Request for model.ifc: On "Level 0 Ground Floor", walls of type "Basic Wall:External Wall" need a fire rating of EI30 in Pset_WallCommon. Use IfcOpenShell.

First a look at what the model holds.

```python
import ifcopenshell
import ifcopenshell.util.element

model = ifcopenshell.open("model.ifc")
print(model.schema)
storey = next(s for s in model.by_type("IfcBuildingStorey") if s.Name == "Level 0 Ground Floor")
walls = [e for e in ifcopenshell.util.element.get_decomposition(storey) if e.is_a("IfcWall")]
seen = {}
for e in walls:
    element_type = ifcopenshell.util.element.get_type(e)
    key = (element_type.Name if element_type != e and element_type else None, ifcopenshell.util.element.get_pset(e, "Pset_WallCommon", "FireRating"))
    seen[key] = seen.get(key, 0) + 1
for (name, value), count in sorted(seen.items(), key=str):
    print(count, "x", name, "|", value)
```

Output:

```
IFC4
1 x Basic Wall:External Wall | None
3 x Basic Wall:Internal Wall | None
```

```python
import ifcopenshell
import ifcopenshell.api.pset
import ifcopenshell.util.element

model = ifcopenshell.open("model.ifc")

storey = next(s for s in model.by_type("IfcBuildingStorey") if s.Name == "Level 0 Ground Floor")
walls = [e for e in ifcopenshell.util.element.get_decomposition(storey) if e.is_a("IfcWall")]

count = 0
for e in walls:
    element_type = ifcopenshell.util.element.get_type(e)
    if element_type in (None, e) or element_type.Name != "Basic Wall:External Wall":
        continue
    # add_pset returns the element's existing set when there is one.
    pset = ifcopenshell.api.pset.add_pset(model, product=e, name="Pset_WallCommon")
    ifcopenshell.api.pset.edit_pset(model, pset=pset, properties={"FireRating": "EI30"})
    count += 1

print(count, "walls updated")

model.write("model_rev.ifc")
```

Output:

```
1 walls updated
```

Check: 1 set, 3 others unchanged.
